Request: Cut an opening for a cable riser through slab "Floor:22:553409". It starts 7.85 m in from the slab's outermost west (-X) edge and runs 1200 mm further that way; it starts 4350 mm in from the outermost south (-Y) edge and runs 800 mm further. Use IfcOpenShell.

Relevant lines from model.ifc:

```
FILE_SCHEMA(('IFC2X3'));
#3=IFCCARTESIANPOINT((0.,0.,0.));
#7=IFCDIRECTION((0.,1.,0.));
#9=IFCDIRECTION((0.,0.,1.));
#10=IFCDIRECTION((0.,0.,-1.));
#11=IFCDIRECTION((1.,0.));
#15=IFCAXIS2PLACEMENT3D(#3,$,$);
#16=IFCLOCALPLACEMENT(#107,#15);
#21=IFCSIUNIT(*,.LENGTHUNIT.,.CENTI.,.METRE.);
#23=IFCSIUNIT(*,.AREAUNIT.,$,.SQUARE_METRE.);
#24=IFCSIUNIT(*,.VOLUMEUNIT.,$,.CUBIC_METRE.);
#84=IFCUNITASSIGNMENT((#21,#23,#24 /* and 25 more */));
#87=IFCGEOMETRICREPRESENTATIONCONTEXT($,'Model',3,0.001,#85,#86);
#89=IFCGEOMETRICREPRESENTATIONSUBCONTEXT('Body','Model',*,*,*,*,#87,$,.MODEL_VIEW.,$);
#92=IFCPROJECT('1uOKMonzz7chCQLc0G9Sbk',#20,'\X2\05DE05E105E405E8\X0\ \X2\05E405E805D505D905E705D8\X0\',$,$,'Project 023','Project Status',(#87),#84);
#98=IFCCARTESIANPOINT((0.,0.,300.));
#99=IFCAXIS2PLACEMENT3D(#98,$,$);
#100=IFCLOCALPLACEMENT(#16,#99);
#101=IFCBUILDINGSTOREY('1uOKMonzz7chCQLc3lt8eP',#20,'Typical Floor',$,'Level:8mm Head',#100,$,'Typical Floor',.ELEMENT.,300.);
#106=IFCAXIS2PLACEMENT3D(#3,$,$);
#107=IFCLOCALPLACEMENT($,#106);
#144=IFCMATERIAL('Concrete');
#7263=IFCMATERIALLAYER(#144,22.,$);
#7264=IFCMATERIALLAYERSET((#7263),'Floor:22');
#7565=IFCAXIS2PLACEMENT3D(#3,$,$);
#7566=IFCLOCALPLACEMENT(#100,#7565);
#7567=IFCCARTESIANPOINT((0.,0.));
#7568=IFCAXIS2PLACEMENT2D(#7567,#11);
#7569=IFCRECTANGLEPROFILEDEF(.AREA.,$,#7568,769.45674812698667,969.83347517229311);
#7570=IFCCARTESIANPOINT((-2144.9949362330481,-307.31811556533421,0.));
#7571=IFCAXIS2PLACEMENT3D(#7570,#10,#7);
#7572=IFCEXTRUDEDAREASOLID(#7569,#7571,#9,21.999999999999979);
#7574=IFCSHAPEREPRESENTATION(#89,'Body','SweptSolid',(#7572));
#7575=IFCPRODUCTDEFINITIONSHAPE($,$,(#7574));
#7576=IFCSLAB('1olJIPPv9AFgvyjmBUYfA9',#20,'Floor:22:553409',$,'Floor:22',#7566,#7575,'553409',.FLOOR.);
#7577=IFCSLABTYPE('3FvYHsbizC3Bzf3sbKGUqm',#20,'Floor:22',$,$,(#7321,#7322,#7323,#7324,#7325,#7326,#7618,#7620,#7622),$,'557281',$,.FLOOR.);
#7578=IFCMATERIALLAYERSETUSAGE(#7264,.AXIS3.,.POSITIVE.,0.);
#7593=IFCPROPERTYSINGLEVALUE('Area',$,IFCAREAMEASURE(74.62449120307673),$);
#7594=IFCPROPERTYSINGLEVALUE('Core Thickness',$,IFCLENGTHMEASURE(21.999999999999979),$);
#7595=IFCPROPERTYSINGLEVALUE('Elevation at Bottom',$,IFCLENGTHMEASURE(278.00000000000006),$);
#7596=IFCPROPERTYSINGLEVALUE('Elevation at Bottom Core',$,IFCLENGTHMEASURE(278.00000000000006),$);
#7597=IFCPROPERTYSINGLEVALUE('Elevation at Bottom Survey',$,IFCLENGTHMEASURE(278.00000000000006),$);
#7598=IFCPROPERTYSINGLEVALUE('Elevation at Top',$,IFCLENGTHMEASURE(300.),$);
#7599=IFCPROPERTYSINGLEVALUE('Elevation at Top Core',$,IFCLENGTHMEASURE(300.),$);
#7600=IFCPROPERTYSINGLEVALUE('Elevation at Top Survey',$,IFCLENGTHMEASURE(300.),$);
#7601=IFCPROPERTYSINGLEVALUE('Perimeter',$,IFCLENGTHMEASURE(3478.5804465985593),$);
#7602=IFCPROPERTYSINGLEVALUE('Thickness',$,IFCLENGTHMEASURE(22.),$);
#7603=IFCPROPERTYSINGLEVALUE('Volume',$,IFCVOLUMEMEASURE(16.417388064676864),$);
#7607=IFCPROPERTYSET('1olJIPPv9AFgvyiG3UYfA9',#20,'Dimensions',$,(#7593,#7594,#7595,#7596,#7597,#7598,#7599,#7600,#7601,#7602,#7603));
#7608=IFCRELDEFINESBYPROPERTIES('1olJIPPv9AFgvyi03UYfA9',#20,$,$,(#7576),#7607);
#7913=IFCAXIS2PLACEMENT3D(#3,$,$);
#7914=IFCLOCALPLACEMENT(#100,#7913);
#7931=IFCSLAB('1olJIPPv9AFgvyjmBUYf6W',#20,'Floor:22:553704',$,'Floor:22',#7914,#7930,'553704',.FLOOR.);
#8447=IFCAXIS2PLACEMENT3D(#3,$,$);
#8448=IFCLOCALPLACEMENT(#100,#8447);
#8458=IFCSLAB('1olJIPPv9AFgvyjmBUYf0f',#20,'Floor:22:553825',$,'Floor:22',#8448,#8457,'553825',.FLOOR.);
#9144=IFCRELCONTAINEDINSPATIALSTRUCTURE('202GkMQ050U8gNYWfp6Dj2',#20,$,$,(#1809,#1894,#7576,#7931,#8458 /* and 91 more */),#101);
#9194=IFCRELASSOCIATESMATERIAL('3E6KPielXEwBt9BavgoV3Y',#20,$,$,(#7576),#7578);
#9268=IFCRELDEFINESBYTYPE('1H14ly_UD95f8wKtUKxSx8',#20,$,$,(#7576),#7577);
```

```python
import numpy as np
import ifcopenshell
import ifcopenshell.api.feature
import ifcopenshell.api.geometry
import ifcopenshell.api.pset
import ifcopenshell.api.root
import ifcopenshell.geom
import ifcopenshell.util.element
import ifcopenshell.util.placement
import ifcopenshell.util.representation
import ifcopenshell.util.shape
import ifcopenshell.util.unit

model = ifcopenshell.open("model.ifc")
unit_scale = ifcopenshell.util.unit.calculate_unit_scale(model)
area_scale = ifcopenshell.util.unit.calculate_unit_scale(model, "AREAUNIT")
volume_scale = ifcopenshell.util.unit.calculate_unit_scale(model, "VOLUMEUNIT")
settings = ifcopenshell.geom.settings()


def volume(element):
    """Net volume in cubic metres, openings subtracted."""
    shape = ifcopenshell.geom.create_shape(settings, element)
    return ifcopenshell.util.shape.get_volume(shape.geometry)


slab = model.by_guid("1olJIPPv9AFgvyjmBUYfA9")
before = volume(slab)

# Extent in the slab's own axes, in metres. The edges named are its -X and -Y sides.
slab_shape = ifcopenshell.geom.create_shape(settings, slab)
vertices = ifcopenshell.util.shape.get_vertices(slab_shape.geometry)
x_min, y_min, bottom = vertices.min(axis=0)
top = vertices[:, 2].max()

opening = ifcopenshell.api.root.create_entity(model, ifc_class="IfcOpeningElement", name="Cable riser opening")
context = ifcopenshell.util.representation.get_context(model, "Model", "Body", "MODEL_VIEW")
width, depth = 1.2, 0.8
outline = [(0.0, 0.0), (width, 0.0), (width, depth), (0.0, depth), (0.0, 0.0)]
# Overshoot both faces by 50 mm so the cut is clean.
shape = ifcopenshell.api.geometry.add_slab_representation(
    model, context=context, depth=top - bottom + 0.1, polyline=outline
)
ifcopenshell.api.geometry.assign_representation(model, product=opening, representation=shape)

matrix = ifcopenshell.util.placement.get_local_placement(slab.ObjectPlacement)
matrix[:, 3] = matrix @ np.append(np.array([x_min + 7.85, y_min + 4.35, bottom - 0.05]) / unit_scale, 1.0)
ifcopenshell.api.geometry.edit_object_placement(model, product=opening, matrix=matrix, is_si=False)
ifcopenshell.api.feature.add_feature(model, feature=opening, element=slab)

after = volume(slab)

# Update the slab's stored quantities.
pset = model.by_id(ifcopenshell.util.element.get_pset(slab, "Dimensions", should_inherit=False)["id"])
ifcopenshell.api.pset.edit_pset(model, pset=pset, properties={
    "Area": model.create_entity("IfcAreaMeasure", after / (top - bottom) / area_scale),
    "Volume": model.create_entity("IfcVolumeMeasure", after / volume_scale),
})

print(f"slab volume {before:.3f} -> {after:.3f} m3")

model.write("model_edited.ifc")
```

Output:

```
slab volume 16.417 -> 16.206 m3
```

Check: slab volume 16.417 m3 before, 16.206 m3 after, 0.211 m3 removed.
